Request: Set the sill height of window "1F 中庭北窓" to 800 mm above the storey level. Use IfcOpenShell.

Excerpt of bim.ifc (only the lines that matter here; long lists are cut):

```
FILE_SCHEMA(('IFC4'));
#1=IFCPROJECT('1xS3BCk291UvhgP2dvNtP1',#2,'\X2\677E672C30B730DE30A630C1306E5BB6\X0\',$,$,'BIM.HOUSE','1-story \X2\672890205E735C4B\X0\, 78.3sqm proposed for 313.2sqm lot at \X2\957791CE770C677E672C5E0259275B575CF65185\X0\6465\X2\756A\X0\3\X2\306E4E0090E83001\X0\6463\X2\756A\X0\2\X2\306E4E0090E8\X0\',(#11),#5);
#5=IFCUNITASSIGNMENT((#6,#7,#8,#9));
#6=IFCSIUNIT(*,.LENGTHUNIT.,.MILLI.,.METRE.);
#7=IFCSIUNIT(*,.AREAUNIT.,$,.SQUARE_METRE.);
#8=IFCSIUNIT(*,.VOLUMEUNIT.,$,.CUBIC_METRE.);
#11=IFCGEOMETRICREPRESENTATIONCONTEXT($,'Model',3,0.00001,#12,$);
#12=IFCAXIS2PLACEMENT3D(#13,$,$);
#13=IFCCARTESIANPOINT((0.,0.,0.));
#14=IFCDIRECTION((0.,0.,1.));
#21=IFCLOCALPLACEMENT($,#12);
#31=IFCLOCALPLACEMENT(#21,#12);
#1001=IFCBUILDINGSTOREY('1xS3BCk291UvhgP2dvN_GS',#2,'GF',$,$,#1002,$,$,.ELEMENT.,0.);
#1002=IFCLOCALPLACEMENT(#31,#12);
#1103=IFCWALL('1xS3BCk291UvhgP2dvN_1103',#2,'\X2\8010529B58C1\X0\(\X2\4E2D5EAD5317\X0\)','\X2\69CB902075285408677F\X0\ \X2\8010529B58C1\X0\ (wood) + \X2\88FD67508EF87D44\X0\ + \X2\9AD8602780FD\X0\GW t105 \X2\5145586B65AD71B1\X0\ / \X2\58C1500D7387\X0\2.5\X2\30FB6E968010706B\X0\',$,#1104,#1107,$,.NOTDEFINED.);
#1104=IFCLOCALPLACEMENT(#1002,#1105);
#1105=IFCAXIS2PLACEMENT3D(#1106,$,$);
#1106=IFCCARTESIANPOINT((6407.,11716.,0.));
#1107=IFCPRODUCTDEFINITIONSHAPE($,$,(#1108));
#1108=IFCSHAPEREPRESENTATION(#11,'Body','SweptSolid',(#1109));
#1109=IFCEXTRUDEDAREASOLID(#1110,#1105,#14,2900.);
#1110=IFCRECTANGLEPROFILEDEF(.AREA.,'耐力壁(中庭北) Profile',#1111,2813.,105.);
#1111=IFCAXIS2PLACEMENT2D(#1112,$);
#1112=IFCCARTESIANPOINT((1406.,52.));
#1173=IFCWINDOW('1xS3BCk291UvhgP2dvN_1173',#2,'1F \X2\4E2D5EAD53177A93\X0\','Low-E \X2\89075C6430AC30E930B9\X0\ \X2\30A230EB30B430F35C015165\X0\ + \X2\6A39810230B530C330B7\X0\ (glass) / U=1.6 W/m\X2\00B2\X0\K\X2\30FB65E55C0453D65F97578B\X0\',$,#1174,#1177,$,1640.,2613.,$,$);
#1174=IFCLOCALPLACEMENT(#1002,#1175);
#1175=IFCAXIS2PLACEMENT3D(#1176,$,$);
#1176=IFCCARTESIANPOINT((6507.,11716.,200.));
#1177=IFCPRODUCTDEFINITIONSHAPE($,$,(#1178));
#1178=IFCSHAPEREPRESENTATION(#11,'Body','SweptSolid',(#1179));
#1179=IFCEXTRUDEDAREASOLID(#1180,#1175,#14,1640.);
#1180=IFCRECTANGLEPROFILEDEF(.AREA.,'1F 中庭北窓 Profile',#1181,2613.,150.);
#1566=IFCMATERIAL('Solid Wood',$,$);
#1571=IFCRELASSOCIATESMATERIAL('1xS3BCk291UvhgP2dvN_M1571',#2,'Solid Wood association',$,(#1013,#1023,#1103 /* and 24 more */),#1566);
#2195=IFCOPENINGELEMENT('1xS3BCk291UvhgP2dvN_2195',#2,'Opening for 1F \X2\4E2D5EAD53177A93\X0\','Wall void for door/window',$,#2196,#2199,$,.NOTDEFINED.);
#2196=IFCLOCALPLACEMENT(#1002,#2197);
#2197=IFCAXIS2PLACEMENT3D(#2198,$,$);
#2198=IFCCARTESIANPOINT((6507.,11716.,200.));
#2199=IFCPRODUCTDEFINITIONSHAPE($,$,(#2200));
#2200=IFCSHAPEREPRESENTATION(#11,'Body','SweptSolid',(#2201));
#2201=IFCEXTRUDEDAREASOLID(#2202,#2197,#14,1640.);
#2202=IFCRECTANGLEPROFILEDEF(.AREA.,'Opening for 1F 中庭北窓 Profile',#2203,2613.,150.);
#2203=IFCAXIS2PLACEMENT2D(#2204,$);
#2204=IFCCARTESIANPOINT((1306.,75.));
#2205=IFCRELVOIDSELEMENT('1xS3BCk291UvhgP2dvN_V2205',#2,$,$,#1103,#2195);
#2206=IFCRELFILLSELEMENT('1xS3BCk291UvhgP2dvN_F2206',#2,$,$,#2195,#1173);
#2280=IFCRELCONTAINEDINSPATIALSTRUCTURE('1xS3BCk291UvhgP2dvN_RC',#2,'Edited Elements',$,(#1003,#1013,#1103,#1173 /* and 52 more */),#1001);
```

```python
import numpy as np
import ifcopenshell
import ifcopenshell.api.geometry
import ifcopenshell.geom
import ifcopenshell.util.element
import ifcopenshell.util.placement
import ifcopenshell.util.shape
import ifcopenshell.util.unit

model = ifcopenshell.open("bim.ifc")
unit_scale = ifcopenshell.util.unit.calculate_unit_scale(model)

window = model.by_guid("1xS3BCk291UvhgP2dvN_1173")
opening = window.FillsVoids[0].RelatingOpeningElement
storey = ifcopenshell.util.element.get_container(window, ifc_class="IfcBuildingStorey")
level = ifcopenshell.util.placement.get_local_placement(storey.ObjectPlacement)[2, 3]

# The opening's origin need not be at the sill, so measure its lowest point.
shape = ifcopenshell.geom.create_shape(ifcopenshell.geom.settings(), opening)
bottom = ifcopenshell.util.shape.get_shape_bottom_elevation(shape, shape.geometry) / unit_scale
dz = level + 800.0 - bottom

shift = np.array([0.0, 0.0, dz])
# The window is not placed relative to its opening, so move both.
for product in (opening, window):
    matrix = ifcopenshell.util.placement.get_local_placement(product.ObjectPlacement)
    matrix[:3, 3] += shift
    ifcopenshell.api.geometry.edit_object_placement(model, product=product, matrix=matrix, is_si=False)

print(f"moved by {dz * unit_scale:+.3f} m")

model.write("bim_rev.ifc")
```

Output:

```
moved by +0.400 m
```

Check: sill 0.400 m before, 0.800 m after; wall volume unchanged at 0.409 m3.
